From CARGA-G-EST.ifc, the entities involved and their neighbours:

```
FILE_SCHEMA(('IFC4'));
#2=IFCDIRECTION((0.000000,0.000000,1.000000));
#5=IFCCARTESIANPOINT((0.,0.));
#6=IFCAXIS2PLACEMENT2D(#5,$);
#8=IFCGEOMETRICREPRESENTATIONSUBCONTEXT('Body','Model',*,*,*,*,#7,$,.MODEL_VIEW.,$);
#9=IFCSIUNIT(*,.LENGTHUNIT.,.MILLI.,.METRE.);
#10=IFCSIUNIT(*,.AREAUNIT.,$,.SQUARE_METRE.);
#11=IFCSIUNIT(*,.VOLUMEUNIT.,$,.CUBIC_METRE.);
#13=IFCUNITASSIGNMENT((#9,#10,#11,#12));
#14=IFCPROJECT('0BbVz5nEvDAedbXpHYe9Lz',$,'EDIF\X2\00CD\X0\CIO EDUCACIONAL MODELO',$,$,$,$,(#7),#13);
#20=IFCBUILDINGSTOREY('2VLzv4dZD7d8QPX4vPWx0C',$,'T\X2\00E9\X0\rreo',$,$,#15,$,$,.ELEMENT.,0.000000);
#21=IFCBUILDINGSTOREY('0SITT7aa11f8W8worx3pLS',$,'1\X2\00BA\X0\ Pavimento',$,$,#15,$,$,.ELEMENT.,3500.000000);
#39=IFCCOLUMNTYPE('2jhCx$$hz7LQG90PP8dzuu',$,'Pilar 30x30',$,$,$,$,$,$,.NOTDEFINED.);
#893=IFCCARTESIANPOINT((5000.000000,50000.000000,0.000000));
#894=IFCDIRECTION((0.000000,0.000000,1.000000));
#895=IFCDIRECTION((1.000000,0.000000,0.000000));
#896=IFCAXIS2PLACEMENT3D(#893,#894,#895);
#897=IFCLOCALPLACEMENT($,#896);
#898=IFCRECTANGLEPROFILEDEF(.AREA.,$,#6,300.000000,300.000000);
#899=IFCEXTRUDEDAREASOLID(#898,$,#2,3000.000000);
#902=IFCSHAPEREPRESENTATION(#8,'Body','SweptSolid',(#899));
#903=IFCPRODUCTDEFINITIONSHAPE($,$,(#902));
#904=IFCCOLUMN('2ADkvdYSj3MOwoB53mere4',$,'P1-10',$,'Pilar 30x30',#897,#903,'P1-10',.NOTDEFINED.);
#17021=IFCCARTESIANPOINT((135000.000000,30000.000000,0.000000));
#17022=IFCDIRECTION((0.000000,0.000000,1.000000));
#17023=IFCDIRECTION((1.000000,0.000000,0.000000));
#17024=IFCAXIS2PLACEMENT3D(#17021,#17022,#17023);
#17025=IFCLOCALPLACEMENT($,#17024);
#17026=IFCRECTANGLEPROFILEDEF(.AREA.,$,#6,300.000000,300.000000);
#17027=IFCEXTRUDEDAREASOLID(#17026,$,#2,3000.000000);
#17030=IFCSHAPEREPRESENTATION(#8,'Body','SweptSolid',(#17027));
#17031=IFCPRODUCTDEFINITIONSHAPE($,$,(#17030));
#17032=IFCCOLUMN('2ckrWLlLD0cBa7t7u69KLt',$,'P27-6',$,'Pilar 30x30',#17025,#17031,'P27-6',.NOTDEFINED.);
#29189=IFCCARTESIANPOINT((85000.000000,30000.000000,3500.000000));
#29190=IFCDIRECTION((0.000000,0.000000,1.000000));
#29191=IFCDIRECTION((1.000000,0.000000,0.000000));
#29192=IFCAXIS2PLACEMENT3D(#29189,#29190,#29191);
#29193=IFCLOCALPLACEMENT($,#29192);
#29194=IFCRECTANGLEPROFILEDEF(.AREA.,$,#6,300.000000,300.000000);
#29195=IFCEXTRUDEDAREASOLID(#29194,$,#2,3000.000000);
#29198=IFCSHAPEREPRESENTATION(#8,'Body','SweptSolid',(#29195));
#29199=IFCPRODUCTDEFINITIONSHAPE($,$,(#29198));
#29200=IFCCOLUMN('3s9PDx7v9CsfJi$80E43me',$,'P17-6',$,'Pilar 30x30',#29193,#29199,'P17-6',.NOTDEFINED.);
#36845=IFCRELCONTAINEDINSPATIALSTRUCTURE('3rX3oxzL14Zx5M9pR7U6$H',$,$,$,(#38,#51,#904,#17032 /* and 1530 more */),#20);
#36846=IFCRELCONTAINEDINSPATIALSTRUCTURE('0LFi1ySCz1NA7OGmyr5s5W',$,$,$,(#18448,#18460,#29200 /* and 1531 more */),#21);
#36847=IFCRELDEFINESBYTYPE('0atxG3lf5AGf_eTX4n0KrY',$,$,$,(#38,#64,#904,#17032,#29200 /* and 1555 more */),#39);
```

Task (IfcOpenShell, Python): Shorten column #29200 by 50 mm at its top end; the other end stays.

```python
import ifcopenshell
import ifcopenshell.util.representation
import ifcopenshell.util.unit

model = ifcopenshell.open("CARGA-G-EST.ifc")
unit_scale = ifcopenshell.util.unit.calculate_unit_scale(model)

member = model.by_id(29200)
change = -0.05 / unit_scale

# The extrusion runs towards the end named, so only its depth changes.
body = ifcopenshell.util.representation.get_representation(member, "Model", "Body")
solid = body.Items[0]
old_length = solid.Depth
solid.Depth += change

print(f"length {old_length:g} -> {solid.Depth:g}")

model.write("CARGA-G-EST_v2.ifc")
```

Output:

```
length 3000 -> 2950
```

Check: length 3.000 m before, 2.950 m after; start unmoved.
